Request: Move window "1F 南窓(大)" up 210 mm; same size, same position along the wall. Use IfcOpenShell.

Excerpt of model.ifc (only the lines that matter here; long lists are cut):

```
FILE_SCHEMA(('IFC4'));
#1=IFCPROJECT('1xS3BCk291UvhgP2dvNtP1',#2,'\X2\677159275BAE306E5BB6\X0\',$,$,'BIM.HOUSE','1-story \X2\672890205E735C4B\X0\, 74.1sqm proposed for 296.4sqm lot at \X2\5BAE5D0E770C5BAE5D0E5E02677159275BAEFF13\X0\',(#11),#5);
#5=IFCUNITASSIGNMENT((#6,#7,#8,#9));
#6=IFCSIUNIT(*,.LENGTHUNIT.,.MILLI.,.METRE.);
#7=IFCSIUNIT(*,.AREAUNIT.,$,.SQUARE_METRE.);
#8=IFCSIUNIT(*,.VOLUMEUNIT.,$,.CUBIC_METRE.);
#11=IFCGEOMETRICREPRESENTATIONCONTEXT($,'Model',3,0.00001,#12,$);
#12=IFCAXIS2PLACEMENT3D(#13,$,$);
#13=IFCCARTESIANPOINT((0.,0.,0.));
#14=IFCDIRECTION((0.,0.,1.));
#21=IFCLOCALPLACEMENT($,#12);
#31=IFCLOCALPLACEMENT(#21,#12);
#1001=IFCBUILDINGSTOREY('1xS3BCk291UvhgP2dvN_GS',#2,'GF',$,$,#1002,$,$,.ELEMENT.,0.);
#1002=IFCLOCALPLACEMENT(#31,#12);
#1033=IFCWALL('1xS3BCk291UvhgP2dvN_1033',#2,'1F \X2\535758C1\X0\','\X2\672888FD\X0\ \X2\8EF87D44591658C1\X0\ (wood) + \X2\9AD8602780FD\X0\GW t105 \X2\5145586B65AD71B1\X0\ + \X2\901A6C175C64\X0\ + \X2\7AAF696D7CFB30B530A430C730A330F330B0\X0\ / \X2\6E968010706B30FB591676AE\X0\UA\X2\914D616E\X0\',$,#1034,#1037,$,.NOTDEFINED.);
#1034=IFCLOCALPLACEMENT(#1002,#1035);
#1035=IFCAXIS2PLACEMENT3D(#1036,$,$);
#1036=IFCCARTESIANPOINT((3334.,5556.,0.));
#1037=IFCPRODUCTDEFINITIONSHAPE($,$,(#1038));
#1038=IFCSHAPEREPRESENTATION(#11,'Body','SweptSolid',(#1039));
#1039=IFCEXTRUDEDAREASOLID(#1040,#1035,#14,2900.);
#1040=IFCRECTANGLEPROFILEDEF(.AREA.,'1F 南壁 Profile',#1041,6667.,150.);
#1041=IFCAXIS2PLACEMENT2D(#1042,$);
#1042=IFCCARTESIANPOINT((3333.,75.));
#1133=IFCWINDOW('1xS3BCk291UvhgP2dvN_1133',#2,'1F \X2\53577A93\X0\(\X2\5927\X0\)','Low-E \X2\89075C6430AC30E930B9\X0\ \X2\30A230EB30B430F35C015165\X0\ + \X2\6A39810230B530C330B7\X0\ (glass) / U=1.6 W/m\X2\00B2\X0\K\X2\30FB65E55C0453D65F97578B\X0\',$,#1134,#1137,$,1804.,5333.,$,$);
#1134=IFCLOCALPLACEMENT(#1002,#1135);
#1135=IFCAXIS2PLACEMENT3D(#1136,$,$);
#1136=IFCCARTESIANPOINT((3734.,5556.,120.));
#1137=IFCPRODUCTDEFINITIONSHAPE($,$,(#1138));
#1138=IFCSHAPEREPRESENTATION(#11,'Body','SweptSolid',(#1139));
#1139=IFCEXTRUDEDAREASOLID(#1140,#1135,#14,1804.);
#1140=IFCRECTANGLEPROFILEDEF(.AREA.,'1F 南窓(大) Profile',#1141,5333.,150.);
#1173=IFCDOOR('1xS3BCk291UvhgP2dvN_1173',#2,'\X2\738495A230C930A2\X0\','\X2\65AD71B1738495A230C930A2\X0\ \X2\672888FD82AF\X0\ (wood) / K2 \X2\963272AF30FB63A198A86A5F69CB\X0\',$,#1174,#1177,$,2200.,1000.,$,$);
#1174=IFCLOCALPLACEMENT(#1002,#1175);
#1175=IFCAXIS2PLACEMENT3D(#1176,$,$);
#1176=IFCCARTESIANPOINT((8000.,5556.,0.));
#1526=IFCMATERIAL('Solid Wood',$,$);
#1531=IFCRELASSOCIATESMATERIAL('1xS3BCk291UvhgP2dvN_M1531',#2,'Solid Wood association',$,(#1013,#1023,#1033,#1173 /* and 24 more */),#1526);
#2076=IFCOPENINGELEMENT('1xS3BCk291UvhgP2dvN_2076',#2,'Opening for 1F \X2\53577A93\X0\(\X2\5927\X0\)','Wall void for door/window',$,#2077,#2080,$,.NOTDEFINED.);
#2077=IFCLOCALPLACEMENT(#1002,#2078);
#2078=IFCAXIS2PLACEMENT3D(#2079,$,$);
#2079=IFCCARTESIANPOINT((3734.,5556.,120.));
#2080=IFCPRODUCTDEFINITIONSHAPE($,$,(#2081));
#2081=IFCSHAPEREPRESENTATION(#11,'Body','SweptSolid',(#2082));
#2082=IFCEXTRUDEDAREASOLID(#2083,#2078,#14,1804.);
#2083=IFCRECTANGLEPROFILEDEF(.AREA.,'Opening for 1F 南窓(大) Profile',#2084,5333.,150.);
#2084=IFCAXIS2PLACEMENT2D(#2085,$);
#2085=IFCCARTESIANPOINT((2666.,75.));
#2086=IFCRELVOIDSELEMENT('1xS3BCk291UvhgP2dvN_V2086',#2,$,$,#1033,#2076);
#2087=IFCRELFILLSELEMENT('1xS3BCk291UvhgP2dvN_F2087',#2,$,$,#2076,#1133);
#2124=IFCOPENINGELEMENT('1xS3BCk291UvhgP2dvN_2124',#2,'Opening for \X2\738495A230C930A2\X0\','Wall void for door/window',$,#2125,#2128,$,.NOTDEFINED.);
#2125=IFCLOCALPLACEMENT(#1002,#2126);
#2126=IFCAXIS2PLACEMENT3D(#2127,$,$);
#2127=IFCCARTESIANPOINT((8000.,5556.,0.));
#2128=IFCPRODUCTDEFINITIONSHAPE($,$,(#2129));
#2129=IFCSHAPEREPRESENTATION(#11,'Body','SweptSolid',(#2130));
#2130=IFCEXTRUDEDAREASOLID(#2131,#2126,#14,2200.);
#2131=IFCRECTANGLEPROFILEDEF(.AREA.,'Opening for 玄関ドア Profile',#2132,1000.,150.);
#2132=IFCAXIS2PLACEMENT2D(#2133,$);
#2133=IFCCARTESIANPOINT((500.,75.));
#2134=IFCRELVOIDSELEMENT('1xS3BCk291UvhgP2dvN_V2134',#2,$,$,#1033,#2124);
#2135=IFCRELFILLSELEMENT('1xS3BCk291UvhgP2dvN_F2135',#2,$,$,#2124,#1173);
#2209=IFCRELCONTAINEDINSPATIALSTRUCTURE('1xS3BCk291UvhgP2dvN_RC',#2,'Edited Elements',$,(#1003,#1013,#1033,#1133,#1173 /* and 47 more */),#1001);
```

```python
import numpy as np
import ifcopenshell
import ifcopenshell.api.geometry
import ifcopenshell.util.placement
import ifcopenshell.util.unit

model = ifcopenshell.open("model.ifc")
unit_scale = ifcopenshell.util.unit.calculate_unit_scale(model)

window = model.by_guid("1xS3BCk291UvhgP2dvN_1133")
opening = window.FillsVoids[0].RelatingOpeningElement
dz = 0.21 / unit_scale

shift = np.array([0.0, 0.0, dz])
# The window is not placed relative to its opening, so move both.
for product in (opening, window):
    matrix = ifcopenshell.util.placement.get_local_placement(product.ObjectPlacement)
    matrix[:3, 3] += shift
    ifcopenshell.api.geometry.edit_object_placement(model, product=product, matrix=matrix, is_si=False)

print(f"moved by {dz * unit_scale:+.3f} m")

model.write("model_edited.ifc")
```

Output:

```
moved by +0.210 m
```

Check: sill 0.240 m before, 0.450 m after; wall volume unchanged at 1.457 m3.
